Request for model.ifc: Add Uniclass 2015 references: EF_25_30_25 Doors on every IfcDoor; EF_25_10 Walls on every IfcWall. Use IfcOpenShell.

First a look at what the model holds.

```python
import ifcopenshell

model = ifcopenshell.open("model.ifc")
print(model.schema)
print("classifications:", [c.Name for c in model.by_type("IfcClassification")])
for ifc_class in ("IfcDoor", "IfcRoof", "IfcStair", "IfcWall", "IfcWindow"):
    print(ifc_class, len(model.by_type(ifc_class)))
```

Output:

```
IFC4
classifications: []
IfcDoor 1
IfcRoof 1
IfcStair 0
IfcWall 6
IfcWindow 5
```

```python
import ifcopenshell
import ifcopenshell.api.classification

model = ifcopenshell.open("model.ifc")

system = ifcopenshell.api.classification.add_classification(model, classification="Uniclass 2015")

codes = {
    "IfcDoor": ("EF_25_30_25", "Doors"),
    "IfcWall": ("EF_25_10", "Walls"),
}
for ifc_class, (code, name) in codes.items():
    products = model.by_type(ifc_class)
    ifcopenshell.api.classification.add_reference(
        model, products=products, classification=system, identification=code, name=name
    )
    print(code, len(products))

model.write("model_edited.ifc")
```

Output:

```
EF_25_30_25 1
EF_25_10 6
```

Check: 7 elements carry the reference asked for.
